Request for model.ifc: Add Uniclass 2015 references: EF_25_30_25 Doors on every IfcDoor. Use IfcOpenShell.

First a look at what the model holds.

```python
import ifcopenshell

model = ifcopenshell.open("model.ifc")
print(model.schema)
print("classifications:", [c.Name for c in model.by_type("IfcClassification")])
for ifc_class in ("IfcDoor", "IfcRoof", "IfcStair", "IfcWall", "IfcWindow"):
    print(ifc_class, len(model.by_type(ifc_class)))
```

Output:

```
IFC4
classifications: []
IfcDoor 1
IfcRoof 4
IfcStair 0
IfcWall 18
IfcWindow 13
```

```python
import ifcopenshell
import ifcopenshell.api.classification

model = ifcopenshell.open("model.ifc")

system = ifcopenshell.api.classification.add_classification(model, classification="Uniclass 2015")

codes = {
    "IfcDoor": ("EF_25_30_25", "Doors"),
}
for ifc_class, (code, name) in codes.items():
    products = model.by_type(ifc_class)
    ifcopenshell.api.classification.add_reference(
        model, products=products, classification=system, identification=code, name=name
    )
    print(code, len(products))

model.write("model-out.ifc")
```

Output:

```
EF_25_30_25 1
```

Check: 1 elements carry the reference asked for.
